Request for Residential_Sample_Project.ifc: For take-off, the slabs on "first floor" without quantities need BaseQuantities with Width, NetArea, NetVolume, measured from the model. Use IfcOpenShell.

First a look at what the model holds.

```python
import ifcopenshell
import ifcopenshell.util.element
import ifcopenshell.util.unit

model = ifcopenshell.open("Residential_Sample_Project.ifc")
print(model.schema)
for unit_type in ("LENGTHUNIT", "AREAUNIT", "VOLUMEUNIT"):
    print(unit_type, ifcopenshell.util.unit.calculate_unit_scale(model, unit_type))
storey = next(s for s in model.by_type("IfcBuildingStorey") if s.Name == "first floor")
slabs = [e for e in ifcopenshell.util.element.get_decomposition(storey) if e.is_a("IfcSlab")]
for e in sorted(slabs, key=lambda e: e.id()):
    print(e.id(), e.is_a(), e.Name, list(ifcopenshell.util.element.get_psets(e, qtos_only=True)), sep=" | ")
```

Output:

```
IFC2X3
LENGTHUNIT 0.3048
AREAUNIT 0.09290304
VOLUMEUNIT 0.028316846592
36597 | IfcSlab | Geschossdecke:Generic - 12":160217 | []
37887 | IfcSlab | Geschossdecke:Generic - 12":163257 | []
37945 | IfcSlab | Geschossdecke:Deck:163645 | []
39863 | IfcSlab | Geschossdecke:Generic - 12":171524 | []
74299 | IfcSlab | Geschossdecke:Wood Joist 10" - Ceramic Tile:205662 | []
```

```python
import ifcopenshell
import ifcopenshell.api.pset
import ifcopenshell.geom
import ifcopenshell.util.element
import ifcopenshell.util.shape
import ifcopenshell.util.unit

model = ifcopenshell.open("Residential_Sample_Project.ifc")
unit_scale = ifcopenshell.util.unit.calculate_unit_scale(model)
area_scale = ifcopenshell.util.unit.calculate_unit_scale(model, "AREAUNIT")
volume_scale = ifcopenshell.util.unit.calculate_unit_scale(model, "VOLUMEUNIT")
settings = ifcopenshell.geom.settings()

storey = next(s for s in model.by_type("IfcBuildingStorey") if s.Name == "first floor")
slabs = [e for e in ifcopenshell.util.element.get_decomposition(storey) if e.is_a("IfcSlab")]

for e in sorted(slabs, key=lambda e: e.id()):
    if ifcopenshell.util.element.get_psets(e, qtos_only=True, should_inherit=False):
        continue
    # Geometry comes back in metres, in the element's own axes.
    shape = ifcopenshell.geom.create_shape(settings, e)
    values = {
        "Width": ifcopenshell.util.shape.get_z(shape.geometry) / unit_scale,
        "NetArea": ifcopenshell.util.shape.get_footprint_area(shape.geometry) / area_scale,
        "NetVolume": ifcopenshell.util.shape.get_volume(shape.geometry) / volume_scale,
    }
    qto = ifcopenshell.api.pset.add_qto(model, product=e, name="BaseQuantities")
    ifcopenshell.api.pset.edit_qto(model, qto=qto, properties=values)
    print(e.id(), {k: round(v, 3) for k, v in values.items()})

model.write("Residential_Sample_Project_v2.ifc")
```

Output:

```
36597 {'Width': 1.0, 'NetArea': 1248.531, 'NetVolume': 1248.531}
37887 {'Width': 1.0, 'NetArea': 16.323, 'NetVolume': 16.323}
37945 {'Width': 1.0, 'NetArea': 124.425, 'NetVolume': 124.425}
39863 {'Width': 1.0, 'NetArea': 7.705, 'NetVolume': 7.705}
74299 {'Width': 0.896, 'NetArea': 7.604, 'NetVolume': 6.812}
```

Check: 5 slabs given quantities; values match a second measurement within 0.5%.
